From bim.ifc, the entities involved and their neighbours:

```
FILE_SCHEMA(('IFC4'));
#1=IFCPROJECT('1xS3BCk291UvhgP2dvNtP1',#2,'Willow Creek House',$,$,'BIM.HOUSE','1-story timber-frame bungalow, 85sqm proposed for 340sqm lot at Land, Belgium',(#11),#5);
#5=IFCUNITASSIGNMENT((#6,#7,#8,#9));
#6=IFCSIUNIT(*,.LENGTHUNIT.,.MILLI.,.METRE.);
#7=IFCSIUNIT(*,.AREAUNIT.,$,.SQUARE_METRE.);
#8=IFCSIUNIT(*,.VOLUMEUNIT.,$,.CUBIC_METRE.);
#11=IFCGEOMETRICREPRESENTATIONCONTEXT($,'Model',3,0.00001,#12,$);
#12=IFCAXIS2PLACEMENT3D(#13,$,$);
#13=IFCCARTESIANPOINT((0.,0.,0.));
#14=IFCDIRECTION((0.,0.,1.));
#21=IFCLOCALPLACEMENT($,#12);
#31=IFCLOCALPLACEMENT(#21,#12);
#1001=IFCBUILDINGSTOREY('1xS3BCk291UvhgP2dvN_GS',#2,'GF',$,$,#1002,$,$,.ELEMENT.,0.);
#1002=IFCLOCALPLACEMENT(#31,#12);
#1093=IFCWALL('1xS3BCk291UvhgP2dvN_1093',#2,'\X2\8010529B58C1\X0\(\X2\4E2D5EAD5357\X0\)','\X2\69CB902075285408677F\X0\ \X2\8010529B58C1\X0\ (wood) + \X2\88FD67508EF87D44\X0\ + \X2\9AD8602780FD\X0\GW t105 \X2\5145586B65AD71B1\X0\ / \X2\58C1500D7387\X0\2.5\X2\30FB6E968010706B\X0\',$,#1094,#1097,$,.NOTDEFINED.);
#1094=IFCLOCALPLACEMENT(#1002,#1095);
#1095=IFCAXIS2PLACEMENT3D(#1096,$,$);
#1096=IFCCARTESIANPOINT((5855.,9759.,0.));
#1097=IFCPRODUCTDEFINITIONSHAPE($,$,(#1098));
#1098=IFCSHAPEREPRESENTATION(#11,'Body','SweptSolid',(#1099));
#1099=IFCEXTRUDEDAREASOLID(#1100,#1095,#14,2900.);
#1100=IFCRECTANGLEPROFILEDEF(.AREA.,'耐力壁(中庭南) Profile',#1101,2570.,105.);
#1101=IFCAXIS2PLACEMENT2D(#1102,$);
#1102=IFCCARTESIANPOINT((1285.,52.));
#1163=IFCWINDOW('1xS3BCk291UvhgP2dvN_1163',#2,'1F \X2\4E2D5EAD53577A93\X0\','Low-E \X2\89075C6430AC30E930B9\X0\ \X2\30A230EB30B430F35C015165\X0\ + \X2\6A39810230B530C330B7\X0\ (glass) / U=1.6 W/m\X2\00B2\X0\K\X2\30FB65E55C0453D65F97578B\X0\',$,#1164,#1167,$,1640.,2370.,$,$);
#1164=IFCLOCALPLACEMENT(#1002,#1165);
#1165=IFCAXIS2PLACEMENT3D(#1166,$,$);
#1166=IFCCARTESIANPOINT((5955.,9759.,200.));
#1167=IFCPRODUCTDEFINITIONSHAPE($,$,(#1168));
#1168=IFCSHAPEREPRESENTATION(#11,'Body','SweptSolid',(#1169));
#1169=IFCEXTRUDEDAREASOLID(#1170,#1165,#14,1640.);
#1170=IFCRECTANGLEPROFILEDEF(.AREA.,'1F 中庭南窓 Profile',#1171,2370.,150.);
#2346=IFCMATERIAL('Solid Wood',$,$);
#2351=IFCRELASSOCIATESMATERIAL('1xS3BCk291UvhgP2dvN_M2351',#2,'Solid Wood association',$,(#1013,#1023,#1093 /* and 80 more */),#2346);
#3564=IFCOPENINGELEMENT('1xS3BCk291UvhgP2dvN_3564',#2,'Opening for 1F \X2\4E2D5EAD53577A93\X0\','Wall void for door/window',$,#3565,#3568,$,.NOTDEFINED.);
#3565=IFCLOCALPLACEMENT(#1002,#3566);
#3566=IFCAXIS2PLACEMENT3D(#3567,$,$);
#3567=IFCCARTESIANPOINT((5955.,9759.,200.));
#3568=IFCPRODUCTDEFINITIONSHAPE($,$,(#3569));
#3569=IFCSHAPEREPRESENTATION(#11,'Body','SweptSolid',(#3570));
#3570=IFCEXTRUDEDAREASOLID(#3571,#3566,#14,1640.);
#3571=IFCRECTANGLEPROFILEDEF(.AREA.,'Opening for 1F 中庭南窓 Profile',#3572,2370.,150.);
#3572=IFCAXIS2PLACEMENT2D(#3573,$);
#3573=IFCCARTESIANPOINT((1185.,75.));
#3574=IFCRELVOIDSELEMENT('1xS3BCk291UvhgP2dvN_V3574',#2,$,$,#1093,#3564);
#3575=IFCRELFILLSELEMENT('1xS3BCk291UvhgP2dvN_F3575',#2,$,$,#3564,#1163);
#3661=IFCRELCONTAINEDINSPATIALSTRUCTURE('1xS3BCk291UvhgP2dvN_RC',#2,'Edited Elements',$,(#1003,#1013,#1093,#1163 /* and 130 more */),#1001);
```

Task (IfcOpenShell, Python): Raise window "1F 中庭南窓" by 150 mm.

```python
import numpy as np
import ifcopenshell
import ifcopenshell.api.geometry
import ifcopenshell.util.placement
import ifcopenshell.util.unit

model = ifcopenshell.open("bim.ifc")
unit_scale = ifcopenshell.util.unit.calculate_unit_scale(model)

window = model.by_guid("1xS3BCk291UvhgP2dvN_1163")
opening = window.FillsVoids[0].RelatingOpeningElement
dz = 150.0

shift = np.array([0.0, 0.0, dz])
# The window is not placed relative to its opening, so move both.
for product in (opening, window):
    matrix = ifcopenshell.util.placement.get_local_placement(product.ObjectPlacement)
    matrix[:3, 3] += shift
    ifcopenshell.api.geometry.edit_object_placement(model, product=product, matrix=matrix, is_si=False)

print(f"moved by {dz * unit_scale:+.3f} m")

model.write("bim_updated.ifc")
```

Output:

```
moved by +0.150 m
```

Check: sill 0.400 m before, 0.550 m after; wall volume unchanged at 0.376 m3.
